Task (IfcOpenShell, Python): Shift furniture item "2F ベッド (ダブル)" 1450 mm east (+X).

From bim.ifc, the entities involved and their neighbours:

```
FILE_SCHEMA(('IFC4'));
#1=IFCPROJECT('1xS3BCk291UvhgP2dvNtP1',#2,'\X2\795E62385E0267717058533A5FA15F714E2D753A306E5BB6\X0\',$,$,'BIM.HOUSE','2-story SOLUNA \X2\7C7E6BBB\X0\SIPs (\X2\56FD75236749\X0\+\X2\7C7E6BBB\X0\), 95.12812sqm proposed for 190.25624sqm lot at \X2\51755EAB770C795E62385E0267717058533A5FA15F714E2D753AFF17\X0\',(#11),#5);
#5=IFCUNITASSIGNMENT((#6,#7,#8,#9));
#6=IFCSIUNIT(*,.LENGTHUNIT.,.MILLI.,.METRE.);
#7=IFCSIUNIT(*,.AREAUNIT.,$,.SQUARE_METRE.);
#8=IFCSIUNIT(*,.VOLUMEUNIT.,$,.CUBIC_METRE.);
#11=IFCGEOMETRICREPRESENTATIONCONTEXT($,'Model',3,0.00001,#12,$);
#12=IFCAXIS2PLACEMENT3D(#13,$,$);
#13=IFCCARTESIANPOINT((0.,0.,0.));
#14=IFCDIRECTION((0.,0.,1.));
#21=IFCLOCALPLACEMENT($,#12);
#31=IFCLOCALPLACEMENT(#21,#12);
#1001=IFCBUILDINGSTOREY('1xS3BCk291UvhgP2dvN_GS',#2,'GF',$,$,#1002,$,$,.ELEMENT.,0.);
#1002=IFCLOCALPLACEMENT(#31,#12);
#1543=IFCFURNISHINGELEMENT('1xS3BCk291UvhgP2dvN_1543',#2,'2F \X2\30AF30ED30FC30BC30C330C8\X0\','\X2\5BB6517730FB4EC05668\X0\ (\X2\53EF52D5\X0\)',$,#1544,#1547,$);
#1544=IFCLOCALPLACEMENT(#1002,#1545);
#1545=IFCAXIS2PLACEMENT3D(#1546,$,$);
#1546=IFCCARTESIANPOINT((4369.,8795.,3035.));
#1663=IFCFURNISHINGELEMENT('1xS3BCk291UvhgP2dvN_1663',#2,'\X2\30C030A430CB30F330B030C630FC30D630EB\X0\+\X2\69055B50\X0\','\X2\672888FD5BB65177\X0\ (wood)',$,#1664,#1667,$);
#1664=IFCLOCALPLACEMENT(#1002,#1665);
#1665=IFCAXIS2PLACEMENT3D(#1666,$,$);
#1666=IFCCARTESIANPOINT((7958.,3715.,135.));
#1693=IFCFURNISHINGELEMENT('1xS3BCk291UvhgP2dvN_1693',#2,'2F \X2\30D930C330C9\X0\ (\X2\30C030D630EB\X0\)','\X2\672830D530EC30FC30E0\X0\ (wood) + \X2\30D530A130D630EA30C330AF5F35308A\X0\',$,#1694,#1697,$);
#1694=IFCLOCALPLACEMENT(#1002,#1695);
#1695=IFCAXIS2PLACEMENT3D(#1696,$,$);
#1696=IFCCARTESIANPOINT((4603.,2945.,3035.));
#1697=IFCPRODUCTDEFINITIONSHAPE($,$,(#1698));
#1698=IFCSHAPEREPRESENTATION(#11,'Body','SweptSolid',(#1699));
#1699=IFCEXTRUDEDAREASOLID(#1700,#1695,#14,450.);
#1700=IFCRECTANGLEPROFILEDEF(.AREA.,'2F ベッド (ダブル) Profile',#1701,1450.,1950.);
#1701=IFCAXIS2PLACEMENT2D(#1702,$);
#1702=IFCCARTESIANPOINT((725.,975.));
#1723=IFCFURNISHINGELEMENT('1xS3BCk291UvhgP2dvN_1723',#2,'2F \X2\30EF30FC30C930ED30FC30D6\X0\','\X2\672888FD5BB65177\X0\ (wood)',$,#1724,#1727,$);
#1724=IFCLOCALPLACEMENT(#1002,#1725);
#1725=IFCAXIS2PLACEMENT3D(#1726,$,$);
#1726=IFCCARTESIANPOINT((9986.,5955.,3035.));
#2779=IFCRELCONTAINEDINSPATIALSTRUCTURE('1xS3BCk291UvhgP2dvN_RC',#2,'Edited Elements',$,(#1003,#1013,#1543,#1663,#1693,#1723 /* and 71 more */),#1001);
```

```python
import ifcopenshell
import ifcopenshell.api.geometry
import ifcopenshell.util.placement
import ifcopenshell.util.unit

model = ifcopenshell.open("bim.ifc")
unit_scale = ifcopenshell.util.unit.calculate_unit_scale(model)

item = model.by_guid("1xS3BCk291UvhgP2dvN_1693")
matrix = ifcopenshell.util.placement.get_local_placement(item.ObjectPlacement)
matrix[0, 3] += 1.45 / unit_scale
ifcopenshell.api.geometry.edit_object_placement(model, product=item, matrix=matrix, is_si=False)

print(ifcopenshell.util.placement.get_local_placement(item.ObjectPlacement).round(3) + 0.0)

model.write("bim_edited.ifc")
```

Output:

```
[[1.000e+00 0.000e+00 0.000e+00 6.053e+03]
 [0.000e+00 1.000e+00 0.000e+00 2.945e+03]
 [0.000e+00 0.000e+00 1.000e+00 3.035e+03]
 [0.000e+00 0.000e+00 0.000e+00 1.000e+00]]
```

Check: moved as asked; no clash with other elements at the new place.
